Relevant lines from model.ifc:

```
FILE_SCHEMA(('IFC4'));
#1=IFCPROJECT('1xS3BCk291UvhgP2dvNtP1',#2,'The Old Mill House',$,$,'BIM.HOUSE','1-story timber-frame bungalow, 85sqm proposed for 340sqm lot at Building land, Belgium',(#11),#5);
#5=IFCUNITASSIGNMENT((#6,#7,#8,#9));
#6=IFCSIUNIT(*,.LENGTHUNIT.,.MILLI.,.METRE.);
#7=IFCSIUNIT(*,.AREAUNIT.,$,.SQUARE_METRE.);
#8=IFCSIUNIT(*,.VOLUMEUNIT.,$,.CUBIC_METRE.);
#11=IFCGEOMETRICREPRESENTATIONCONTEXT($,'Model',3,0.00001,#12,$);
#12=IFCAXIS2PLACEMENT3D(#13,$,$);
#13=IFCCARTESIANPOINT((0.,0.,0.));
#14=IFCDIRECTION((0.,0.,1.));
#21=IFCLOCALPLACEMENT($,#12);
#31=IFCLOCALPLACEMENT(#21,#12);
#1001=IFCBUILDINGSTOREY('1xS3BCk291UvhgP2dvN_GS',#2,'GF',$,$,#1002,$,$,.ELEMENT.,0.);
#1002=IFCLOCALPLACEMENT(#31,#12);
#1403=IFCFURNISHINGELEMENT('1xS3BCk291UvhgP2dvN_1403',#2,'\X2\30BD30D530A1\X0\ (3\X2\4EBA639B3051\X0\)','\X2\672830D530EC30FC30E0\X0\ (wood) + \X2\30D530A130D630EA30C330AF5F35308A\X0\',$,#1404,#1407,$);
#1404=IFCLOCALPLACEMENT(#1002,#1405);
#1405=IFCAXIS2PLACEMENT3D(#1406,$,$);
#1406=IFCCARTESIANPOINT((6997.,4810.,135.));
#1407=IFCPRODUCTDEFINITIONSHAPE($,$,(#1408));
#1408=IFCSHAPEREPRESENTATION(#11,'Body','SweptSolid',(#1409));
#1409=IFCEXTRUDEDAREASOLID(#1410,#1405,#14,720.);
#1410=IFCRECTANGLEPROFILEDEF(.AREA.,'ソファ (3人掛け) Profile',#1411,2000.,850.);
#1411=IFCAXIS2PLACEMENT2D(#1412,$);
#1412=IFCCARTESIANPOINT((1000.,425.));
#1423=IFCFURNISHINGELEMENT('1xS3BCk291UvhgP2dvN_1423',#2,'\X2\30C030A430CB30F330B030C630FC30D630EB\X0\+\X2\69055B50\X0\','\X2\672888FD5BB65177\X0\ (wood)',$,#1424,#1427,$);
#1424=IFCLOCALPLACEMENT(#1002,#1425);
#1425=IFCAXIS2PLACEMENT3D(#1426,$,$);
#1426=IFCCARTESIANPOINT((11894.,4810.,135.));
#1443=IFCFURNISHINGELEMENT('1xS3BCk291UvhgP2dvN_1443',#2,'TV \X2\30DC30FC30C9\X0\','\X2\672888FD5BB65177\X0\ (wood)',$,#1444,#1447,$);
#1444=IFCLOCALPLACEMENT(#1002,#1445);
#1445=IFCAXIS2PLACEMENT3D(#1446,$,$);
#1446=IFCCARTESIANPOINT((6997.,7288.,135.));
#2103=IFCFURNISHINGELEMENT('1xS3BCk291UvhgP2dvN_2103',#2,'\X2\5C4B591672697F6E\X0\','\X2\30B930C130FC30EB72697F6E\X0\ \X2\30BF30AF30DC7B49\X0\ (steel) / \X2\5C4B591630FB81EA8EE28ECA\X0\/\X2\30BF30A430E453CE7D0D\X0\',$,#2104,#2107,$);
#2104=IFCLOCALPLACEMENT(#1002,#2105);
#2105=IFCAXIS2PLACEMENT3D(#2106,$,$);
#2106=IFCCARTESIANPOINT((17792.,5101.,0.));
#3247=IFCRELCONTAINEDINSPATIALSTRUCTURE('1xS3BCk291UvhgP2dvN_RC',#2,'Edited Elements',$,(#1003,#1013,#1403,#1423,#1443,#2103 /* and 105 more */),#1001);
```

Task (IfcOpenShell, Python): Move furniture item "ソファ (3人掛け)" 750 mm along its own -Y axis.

```python
import ifcopenshell
import ifcopenshell.api.geometry
import ifcopenshell.util.placement
import ifcopenshell.util.unit

model = ifcopenshell.open("model.ifc")
unit_scale = ifcopenshell.util.unit.calculate_unit_scale(model)

item = model.by_guid("1xS3BCk291UvhgP2dvN_1403")
matrix = ifcopenshell.util.placement.get_local_placement(item.ObjectPlacement)
matrix[:3, 3] -= matrix[:3, 1] * 0.75 / unit_scale
ifcopenshell.api.geometry.edit_object_placement(model, product=item, matrix=matrix, is_si=False)

print(ifcopenshell.util.placement.get_local_placement(item.ObjectPlacement).round(3) + 0.0)

model.write("model_updated.ifc")
```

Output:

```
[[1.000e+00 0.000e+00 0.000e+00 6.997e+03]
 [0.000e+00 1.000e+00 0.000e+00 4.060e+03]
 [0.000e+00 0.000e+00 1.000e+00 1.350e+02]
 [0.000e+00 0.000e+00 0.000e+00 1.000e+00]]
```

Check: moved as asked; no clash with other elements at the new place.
